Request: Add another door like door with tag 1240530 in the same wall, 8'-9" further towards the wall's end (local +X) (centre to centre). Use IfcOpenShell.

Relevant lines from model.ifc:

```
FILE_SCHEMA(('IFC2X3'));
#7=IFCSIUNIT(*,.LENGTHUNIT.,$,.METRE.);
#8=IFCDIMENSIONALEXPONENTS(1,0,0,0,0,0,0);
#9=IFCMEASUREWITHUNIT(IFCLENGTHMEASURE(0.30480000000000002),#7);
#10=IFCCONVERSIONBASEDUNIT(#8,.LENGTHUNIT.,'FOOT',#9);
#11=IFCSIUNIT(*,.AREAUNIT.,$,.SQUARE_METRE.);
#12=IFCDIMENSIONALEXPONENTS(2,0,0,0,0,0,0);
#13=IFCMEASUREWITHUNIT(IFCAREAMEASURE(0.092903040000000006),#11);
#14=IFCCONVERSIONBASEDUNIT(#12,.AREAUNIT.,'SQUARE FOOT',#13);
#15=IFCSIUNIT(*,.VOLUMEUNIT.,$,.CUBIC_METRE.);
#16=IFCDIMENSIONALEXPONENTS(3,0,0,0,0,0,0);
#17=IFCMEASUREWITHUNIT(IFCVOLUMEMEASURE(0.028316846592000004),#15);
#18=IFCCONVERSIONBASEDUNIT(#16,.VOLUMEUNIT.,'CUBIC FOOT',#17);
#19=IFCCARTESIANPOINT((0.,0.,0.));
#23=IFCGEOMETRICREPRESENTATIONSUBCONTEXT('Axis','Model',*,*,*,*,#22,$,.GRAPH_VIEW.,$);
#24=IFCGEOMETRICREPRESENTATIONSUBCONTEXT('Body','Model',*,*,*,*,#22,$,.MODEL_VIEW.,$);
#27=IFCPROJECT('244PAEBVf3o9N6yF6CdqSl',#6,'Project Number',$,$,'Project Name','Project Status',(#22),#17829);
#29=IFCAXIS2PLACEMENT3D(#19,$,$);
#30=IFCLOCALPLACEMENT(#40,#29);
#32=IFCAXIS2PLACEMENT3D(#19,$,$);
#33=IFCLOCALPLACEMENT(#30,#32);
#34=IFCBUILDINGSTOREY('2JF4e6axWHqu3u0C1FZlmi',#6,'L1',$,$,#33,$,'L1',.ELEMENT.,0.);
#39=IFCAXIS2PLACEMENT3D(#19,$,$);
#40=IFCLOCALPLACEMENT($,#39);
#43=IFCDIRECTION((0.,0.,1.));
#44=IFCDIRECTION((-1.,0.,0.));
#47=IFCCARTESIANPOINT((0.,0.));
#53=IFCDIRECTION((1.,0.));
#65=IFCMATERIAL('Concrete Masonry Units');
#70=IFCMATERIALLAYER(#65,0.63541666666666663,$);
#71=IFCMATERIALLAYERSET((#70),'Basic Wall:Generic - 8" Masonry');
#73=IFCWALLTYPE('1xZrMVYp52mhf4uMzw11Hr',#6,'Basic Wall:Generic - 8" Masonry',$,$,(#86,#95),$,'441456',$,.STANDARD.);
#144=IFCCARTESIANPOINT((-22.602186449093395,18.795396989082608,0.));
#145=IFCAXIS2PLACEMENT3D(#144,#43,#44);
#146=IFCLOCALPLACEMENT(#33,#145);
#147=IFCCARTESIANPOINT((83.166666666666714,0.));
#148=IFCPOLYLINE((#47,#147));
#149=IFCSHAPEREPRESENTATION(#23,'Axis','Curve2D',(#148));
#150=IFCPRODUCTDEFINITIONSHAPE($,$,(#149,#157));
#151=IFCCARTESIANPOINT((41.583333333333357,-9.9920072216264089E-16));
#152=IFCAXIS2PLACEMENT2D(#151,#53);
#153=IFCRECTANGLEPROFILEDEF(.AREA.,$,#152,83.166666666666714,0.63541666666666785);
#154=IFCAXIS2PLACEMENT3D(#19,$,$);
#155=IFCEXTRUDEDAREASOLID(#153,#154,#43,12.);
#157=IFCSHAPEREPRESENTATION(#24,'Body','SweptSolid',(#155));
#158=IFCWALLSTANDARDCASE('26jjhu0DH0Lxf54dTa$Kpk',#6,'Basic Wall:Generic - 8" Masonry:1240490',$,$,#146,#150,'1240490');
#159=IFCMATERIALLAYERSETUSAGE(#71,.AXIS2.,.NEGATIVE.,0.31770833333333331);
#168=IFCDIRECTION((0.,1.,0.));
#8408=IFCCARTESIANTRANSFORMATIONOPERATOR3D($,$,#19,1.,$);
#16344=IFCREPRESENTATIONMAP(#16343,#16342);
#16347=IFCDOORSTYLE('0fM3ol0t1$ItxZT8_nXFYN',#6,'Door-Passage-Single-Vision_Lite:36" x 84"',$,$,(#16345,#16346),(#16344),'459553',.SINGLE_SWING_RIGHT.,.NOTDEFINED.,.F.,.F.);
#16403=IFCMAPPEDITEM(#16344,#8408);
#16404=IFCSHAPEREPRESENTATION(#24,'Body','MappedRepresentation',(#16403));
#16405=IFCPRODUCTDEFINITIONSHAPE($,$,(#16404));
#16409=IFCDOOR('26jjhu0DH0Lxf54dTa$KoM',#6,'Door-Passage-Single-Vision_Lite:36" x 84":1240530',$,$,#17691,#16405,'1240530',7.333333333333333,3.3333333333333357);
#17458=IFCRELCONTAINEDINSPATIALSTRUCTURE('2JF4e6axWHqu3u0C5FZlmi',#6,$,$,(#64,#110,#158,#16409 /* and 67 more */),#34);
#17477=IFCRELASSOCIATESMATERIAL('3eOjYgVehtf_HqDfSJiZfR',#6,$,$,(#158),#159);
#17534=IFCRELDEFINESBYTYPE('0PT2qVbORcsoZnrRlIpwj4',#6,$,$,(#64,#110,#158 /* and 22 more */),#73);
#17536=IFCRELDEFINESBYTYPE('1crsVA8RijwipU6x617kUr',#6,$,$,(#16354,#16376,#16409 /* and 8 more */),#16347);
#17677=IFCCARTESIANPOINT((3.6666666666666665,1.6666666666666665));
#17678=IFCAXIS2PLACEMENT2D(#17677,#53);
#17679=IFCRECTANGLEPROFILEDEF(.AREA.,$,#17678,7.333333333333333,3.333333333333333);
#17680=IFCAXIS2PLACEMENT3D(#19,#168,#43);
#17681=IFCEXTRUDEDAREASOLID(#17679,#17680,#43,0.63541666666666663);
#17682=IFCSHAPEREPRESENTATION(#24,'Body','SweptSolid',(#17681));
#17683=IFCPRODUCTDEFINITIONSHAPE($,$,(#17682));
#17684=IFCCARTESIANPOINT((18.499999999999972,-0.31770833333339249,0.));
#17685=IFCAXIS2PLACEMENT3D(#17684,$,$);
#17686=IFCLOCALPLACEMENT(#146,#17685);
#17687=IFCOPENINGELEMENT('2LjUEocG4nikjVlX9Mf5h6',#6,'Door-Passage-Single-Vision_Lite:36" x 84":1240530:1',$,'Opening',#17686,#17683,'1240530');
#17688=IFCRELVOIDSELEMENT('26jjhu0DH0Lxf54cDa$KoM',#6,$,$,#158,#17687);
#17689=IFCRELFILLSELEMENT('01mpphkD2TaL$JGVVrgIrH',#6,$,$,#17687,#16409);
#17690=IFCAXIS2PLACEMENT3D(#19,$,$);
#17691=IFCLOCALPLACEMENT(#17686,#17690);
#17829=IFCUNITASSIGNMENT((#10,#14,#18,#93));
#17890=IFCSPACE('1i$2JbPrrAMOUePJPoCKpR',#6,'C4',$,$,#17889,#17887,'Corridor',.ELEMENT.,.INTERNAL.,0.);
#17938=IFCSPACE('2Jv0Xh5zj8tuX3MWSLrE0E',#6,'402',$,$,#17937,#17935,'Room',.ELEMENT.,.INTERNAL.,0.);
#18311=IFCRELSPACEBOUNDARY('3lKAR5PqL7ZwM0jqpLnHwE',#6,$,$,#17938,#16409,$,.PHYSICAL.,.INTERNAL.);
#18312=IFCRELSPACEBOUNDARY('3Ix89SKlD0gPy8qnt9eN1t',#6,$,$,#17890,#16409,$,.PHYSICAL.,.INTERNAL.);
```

```python
import ifcopenshell
import ifcopenshell.api.feature
import ifcopenshell.api.geometry
import ifcopenshell.api.root
import ifcopenshell.geom
import ifcopenshell.util.element
import ifcopenshell.util.placement
import ifcopenshell.util.shape
import ifcopenshell.util.unit

model = ifcopenshell.open("model.ifc")
unit_scale = ifcopenshell.util.unit.calculate_unit_scale(model)
settings = ifcopenshell.geom.settings()


def volume(element):
    """Net volume in cubic metres, openings subtracted."""
    shape = ifcopenshell.geom.create_shape(settings, element)
    return ifcopenshell.util.shape.get_volume(shape.geometry)


def reuse_history(source, copy):
    """copy_class also copies each property set's owner history, people and application; keep the originals."""
    for rel in copy.IsDefinedBy:
        if rel.is_a("IfcRelDefinesByProperties") and (history := rel.RelatingPropertyDefinition.OwnerHistory):
            rel.RelatingPropertyDefinition.OwnerHistory = source.OwnerHistory
            ifcopenshell.util.element.remove_deep2(model, history)


door = model.by_id(16409)
opening = door.FillsVoids[0].RelatingOpeningElement
wall = opening.VoidsElements[0].RelatingBuildingElement
before = volume(wall)
shift = ifcopenshell.util.placement.get_local_placement(wall.ObjectPlacement)[:3, 0] * 105 * 0.0254 / unit_scale

# copy_class copies the void relationship, type, container and properties, but no geometry.
new_opening = ifcopenshell.api.root.copy_class(model, product=opening)
new_opening.Representation = ifcopenshell.util.element.copy_deep(
    model, opening.Representation, exclude=["IfcGeometricRepresentationContext", "IfcRepresentationMap"]
)
new_opening.Name = 'Door-Passage-Single-Vision_Lite:36" x 84"'
new_opening.Tag = None
new_door = ifcopenshell.api.root.copy_class(model, product=door)
new_door.Representation = ifcopenshell.util.element.copy_deep(
    model, door.Representation, exclude=["IfcGeometricRepresentationContext", "IfcRepresentationMap"]
)
new_door.Name = 'Door-Passage-Single-Vision_Lite:36" x 84"'
new_door.Tag = None
reuse_history(door, new_door)
fills = ifcopenshell.api.feature.add_filling(model, opening=new_opening, element=new_door)
fills.OwnerHistory = new_door.OwnerHistory  # required in IFC2X3

for old, new in ((opening, new_opening), (door, new_door)):
    matrix = ifcopenshell.util.placement.get_local_placement(old.ObjectPlacement)
    matrix[:3, 3] += shift
    ifcopenshell.api.geometry.edit_object_placement(model, product=new, matrix=matrix, is_si=False)

after = volume(wall)

print(f"wall volume {before:.3f} -> {after:.3f} m3")

model.write("model_v2.ifc")
```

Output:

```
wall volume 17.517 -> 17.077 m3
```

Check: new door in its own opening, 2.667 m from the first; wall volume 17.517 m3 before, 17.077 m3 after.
